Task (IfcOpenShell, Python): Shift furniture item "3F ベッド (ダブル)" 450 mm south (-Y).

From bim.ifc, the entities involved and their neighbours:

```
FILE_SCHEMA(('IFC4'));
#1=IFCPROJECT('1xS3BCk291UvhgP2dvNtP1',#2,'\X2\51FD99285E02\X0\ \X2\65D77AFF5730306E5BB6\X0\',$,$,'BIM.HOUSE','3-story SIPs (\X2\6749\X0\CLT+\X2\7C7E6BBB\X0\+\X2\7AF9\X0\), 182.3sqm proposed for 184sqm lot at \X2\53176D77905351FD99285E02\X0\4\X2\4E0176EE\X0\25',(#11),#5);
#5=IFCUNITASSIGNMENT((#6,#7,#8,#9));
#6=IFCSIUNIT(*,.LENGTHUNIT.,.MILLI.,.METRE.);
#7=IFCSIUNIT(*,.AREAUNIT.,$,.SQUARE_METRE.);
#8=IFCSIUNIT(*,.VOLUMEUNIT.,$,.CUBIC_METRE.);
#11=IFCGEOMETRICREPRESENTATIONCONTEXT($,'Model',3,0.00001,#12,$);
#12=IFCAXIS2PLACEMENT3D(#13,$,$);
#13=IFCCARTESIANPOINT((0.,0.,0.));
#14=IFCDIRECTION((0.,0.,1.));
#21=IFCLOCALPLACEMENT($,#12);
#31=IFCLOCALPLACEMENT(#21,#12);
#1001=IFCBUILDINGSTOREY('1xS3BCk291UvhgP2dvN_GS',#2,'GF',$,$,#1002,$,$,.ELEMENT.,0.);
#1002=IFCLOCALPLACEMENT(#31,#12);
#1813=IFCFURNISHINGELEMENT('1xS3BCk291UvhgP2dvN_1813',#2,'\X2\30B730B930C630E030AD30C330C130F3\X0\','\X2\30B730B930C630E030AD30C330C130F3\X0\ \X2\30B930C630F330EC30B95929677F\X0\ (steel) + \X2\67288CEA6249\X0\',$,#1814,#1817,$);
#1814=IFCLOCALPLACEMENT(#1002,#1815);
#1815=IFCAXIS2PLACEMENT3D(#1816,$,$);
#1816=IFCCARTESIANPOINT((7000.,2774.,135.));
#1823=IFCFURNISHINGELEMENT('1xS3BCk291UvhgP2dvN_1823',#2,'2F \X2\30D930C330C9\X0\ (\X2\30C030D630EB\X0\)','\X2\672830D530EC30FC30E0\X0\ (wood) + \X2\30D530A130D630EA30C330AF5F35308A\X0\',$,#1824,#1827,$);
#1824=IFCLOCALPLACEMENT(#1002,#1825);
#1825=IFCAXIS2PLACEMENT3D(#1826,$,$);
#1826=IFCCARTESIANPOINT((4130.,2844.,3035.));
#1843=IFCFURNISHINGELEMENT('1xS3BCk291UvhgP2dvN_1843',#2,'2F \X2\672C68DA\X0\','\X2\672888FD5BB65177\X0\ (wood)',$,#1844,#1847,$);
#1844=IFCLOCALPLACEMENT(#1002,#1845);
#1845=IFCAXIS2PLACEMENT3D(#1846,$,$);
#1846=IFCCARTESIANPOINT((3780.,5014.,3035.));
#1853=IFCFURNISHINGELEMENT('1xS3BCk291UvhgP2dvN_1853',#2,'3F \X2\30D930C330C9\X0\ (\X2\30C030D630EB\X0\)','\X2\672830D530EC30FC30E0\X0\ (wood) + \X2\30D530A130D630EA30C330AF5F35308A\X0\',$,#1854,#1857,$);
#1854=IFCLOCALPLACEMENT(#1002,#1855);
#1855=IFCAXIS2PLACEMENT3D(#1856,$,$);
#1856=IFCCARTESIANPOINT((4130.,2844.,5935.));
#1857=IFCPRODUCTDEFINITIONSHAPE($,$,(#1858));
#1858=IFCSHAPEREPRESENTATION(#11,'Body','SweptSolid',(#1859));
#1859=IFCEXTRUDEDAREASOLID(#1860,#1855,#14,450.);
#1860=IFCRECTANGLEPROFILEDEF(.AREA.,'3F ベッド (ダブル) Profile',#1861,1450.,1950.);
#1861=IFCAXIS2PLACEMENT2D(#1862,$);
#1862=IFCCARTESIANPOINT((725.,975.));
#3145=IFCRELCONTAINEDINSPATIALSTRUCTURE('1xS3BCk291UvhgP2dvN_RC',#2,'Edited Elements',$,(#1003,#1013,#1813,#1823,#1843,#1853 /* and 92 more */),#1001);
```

```python
import ifcopenshell
import ifcopenshell.api.geometry
import ifcopenshell.util.placement
import ifcopenshell.util.unit

model = ifcopenshell.open("bim.ifc")
unit_scale = ifcopenshell.util.unit.calculate_unit_scale(model)

item = model.by_guid("1xS3BCk291UvhgP2dvN_1853")
matrix = ifcopenshell.util.placement.get_local_placement(item.ObjectPlacement)
matrix[1, 3] -= 0.45 / unit_scale
ifcopenshell.api.geometry.edit_object_placement(model, product=item, matrix=matrix, is_si=False)

print(ifcopenshell.util.placement.get_local_placement(item.ObjectPlacement).round(3) + 0.0)

model.write("bim_v2.ifc")
```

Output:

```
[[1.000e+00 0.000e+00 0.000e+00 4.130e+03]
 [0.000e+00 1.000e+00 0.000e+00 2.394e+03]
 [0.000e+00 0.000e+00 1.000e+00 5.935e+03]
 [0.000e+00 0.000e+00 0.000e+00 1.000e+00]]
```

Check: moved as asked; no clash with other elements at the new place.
